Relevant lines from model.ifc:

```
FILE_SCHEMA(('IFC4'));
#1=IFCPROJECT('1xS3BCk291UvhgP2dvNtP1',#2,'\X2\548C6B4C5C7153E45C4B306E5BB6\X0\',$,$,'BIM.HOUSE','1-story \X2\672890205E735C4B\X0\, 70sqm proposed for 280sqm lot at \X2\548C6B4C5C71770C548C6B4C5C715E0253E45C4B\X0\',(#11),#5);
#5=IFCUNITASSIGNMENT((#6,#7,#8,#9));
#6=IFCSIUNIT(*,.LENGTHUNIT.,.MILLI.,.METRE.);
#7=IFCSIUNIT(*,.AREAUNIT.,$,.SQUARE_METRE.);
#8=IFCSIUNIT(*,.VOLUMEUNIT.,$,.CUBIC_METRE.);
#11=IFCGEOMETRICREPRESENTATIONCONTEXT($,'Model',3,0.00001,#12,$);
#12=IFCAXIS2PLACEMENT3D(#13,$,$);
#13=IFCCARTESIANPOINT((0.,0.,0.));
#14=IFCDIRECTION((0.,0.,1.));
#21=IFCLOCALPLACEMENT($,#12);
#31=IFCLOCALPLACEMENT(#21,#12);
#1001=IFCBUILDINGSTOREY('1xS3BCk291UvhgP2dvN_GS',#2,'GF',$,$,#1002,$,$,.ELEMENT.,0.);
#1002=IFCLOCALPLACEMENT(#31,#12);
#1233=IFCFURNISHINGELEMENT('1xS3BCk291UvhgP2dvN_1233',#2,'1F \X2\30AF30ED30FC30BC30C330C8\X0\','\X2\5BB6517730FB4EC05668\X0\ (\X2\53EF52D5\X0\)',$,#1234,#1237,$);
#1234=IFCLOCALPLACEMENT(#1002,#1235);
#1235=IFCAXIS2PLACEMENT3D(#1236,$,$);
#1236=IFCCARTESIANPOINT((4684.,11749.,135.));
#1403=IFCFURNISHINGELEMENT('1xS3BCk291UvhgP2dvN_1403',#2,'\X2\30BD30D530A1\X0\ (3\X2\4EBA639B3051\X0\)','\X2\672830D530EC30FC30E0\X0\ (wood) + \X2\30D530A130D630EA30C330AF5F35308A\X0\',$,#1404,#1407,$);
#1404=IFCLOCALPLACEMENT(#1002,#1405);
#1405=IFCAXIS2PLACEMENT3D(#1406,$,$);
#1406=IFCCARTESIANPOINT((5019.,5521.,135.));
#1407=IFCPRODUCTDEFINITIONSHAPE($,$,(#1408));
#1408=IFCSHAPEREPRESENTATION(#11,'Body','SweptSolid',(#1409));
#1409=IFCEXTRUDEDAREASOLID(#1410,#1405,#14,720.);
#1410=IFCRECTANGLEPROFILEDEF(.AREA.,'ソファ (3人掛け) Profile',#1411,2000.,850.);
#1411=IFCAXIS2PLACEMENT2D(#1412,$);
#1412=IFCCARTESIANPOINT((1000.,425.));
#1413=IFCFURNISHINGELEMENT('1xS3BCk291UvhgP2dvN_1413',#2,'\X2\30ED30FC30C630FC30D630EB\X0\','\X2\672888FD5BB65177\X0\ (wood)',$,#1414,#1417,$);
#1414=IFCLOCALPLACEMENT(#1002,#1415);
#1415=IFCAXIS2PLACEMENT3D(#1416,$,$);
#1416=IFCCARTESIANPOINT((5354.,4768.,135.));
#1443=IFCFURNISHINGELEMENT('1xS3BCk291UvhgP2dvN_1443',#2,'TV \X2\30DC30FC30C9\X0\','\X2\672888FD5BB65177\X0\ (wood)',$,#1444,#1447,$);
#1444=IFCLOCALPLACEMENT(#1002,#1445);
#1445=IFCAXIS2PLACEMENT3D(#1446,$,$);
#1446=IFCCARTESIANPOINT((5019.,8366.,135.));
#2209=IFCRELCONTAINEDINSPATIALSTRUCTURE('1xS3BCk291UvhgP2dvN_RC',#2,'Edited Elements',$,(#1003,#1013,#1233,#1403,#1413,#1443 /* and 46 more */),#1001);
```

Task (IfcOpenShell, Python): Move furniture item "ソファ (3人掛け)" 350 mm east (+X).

```python
import ifcopenshell
import ifcopenshell.api.geometry
import ifcopenshell.util.placement
import ifcopenshell.util.unit

model = ifcopenshell.open("model.ifc")
unit_scale = ifcopenshell.util.unit.calculate_unit_scale(model)

item = model.by_guid("1xS3BCk291UvhgP2dvN_1403")
matrix = ifcopenshell.util.placement.get_local_placement(item.ObjectPlacement)
matrix[0, 3] += 0.35 / unit_scale
ifcopenshell.api.geometry.edit_object_placement(model, product=item, matrix=matrix, is_si=False)

print(ifcopenshell.util.placement.get_local_placement(item.ObjectPlacement).round(3) + 0.0)

model.write("model_rev.ifc")
```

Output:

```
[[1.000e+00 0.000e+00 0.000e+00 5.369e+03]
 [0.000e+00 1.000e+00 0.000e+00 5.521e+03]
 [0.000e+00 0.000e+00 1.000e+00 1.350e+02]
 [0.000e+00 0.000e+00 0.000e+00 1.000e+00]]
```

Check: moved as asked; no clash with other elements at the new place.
